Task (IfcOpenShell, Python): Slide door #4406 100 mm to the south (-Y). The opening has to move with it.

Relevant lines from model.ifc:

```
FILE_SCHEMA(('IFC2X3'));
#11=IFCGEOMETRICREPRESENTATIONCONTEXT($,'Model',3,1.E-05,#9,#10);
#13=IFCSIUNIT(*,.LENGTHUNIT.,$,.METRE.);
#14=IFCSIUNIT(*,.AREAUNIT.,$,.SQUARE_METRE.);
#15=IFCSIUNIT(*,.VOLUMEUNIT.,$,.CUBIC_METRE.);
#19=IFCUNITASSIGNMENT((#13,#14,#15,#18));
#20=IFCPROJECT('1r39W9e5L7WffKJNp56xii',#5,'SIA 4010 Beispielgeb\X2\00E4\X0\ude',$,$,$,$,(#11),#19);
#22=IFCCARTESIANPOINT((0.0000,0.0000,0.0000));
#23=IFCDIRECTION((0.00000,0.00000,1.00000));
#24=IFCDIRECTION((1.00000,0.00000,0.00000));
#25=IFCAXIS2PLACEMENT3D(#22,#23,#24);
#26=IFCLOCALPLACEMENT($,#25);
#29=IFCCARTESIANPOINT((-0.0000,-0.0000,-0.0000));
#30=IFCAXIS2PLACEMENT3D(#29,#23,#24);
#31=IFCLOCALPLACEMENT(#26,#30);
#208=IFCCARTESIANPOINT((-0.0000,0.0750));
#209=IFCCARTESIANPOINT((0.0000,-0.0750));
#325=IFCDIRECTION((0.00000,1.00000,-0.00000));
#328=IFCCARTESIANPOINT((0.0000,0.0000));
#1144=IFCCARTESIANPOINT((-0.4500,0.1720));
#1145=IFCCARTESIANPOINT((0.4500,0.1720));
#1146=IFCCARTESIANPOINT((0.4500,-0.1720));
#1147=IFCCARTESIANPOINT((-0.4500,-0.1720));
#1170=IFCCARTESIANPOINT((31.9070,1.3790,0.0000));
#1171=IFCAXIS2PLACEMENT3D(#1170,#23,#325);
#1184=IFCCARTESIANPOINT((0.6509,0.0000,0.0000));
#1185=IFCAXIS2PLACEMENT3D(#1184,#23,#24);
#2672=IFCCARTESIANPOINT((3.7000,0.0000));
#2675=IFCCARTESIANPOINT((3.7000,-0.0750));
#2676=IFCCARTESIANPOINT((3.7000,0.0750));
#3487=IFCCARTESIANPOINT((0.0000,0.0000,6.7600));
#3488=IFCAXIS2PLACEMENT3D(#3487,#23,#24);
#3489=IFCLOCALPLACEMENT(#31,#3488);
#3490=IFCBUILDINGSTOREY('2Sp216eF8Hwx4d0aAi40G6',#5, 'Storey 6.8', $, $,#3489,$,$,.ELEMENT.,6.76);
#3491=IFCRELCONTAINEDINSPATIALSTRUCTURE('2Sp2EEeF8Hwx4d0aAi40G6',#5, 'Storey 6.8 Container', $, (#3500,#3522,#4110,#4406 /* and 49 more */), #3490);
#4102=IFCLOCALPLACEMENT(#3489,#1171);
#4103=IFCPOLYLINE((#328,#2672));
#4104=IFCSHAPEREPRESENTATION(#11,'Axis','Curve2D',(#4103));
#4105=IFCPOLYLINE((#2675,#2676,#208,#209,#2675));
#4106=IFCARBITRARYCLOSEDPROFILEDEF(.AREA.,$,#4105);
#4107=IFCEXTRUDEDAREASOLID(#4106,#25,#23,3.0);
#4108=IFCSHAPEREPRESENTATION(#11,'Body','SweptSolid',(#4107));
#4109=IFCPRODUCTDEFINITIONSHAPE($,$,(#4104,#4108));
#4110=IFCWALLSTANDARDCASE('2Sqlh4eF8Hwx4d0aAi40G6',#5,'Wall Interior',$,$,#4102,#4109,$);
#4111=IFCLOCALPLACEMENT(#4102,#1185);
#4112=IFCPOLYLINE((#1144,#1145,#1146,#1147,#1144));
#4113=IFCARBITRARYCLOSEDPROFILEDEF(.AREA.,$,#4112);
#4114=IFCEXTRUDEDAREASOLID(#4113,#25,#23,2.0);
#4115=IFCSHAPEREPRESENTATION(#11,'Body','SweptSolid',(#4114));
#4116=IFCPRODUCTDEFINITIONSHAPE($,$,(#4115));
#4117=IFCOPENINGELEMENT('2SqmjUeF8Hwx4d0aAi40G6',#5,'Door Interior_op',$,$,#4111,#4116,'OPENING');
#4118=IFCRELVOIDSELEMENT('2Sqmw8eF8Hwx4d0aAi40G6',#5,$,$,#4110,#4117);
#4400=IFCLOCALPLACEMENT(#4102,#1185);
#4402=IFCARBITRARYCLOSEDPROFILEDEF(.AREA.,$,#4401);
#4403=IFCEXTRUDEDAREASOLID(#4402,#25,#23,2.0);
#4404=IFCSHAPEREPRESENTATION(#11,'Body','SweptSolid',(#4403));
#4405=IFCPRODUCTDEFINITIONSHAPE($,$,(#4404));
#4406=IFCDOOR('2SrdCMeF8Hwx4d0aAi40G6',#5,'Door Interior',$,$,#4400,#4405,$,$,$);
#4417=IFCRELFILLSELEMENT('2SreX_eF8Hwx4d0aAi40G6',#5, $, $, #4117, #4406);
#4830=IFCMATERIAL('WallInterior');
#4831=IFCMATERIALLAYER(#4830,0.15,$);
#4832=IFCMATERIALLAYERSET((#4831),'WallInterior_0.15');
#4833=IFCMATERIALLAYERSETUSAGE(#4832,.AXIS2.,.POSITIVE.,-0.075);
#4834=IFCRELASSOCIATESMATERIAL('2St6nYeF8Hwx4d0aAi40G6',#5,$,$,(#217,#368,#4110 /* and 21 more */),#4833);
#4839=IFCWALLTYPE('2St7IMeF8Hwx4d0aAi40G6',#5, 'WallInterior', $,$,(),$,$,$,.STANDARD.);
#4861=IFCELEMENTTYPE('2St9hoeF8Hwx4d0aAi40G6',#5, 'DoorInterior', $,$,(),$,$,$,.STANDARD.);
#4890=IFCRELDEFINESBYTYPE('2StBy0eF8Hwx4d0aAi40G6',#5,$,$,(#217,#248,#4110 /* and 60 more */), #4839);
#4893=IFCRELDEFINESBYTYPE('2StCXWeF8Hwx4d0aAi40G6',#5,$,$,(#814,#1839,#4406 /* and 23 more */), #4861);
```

```python
import ifcopenshell
import ifcopenshell.api.geometry
import ifcopenshell.util.placement

model = ifcopenshell.open("model.ifc")

door = model.by_id(4406)
opening = door.FillsVoids[0].RelatingOpeningElement
wall = opening.VoidsElements[0].RelatingBuildingElement

wall_matrix = ifcopenshell.util.placement.get_local_placement(wall.ObjectPlacement)
shift = wall_matrix[:3, 0] * -0.1
before = ifcopenshell.util.placement.get_local_placement(door.ObjectPlacement)[:3, 3].copy()

# The door is not placed relative to its opening, so move both.
for product in (opening, door):
    matrix = ifcopenshell.util.placement.get_local_placement(product.ObjectPlacement)
    matrix[:3, 3] += shift
    ifcopenshell.api.geometry.edit_object_placement(model, product=product, matrix=matrix, is_si=False)

after = ifcopenshell.util.placement.get_local_placement(door.ObjectPlacement)[:3, 3]
print("door moved by", (after - before).round(3) + 0.0)

model.write("model_updated.ifc")
```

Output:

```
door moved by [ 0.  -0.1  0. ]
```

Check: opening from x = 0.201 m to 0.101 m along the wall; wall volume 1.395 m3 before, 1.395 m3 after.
